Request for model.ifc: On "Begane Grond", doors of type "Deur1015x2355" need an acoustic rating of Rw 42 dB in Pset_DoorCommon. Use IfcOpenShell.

First a look at what the model holds.

```python
import ifcopenshell
import ifcopenshell.util.element

model = ifcopenshell.open("model.ifc")
print(model.schema)
storey = next(s for s in model.by_type("IfcBuildingStorey") if s.Name == "Begane Grond")
doors = [e for e in ifcopenshell.util.element.get_decomposition(storey) if e.is_a("IfcDoor")]
seen = {}
for e in doors:
    element_type = ifcopenshell.util.element.get_type(e)
    key = (element_type.Name if element_type != e and element_type else None, ifcopenshell.util.element.get_pset(e, "Pset_DoorCommon", "AcousticRating"))
    seen[key] = seen.get(key, 0) + 1
for (name, value), count in sorted(seen.items(), key=str):
    print(count, "x", name, "|", value)
```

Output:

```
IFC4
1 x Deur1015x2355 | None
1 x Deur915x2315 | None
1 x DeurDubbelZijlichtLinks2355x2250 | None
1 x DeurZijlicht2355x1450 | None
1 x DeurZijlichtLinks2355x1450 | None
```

```python
import ifcopenshell
import ifcopenshell.api.pset
import ifcopenshell.util.element

model = ifcopenshell.open("model.ifc")

storey = next(s for s in model.by_type("IfcBuildingStorey") if s.Name == "Begane Grond")
doors = [e for e in ifcopenshell.util.element.get_decomposition(storey) if e.is_a("IfcDoor")]

count = 0
for e in doors:
    element_type = ifcopenshell.util.element.get_type(e)
    if element_type in (None, e) or element_type.Name != "Deur1015x2355":
        continue
    # add_pset returns the element's existing set when there is one.
    pset = ifcopenshell.api.pset.add_pset(model, product=e, name="Pset_DoorCommon")
    ifcopenshell.api.pset.edit_pset(model, pset=pset, properties={"AcousticRating": "Rw 42 dB"})
    count += 1

print(count, "doors updated")

model.write("model_edited.ifc")
```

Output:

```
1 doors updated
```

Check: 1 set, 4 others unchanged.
